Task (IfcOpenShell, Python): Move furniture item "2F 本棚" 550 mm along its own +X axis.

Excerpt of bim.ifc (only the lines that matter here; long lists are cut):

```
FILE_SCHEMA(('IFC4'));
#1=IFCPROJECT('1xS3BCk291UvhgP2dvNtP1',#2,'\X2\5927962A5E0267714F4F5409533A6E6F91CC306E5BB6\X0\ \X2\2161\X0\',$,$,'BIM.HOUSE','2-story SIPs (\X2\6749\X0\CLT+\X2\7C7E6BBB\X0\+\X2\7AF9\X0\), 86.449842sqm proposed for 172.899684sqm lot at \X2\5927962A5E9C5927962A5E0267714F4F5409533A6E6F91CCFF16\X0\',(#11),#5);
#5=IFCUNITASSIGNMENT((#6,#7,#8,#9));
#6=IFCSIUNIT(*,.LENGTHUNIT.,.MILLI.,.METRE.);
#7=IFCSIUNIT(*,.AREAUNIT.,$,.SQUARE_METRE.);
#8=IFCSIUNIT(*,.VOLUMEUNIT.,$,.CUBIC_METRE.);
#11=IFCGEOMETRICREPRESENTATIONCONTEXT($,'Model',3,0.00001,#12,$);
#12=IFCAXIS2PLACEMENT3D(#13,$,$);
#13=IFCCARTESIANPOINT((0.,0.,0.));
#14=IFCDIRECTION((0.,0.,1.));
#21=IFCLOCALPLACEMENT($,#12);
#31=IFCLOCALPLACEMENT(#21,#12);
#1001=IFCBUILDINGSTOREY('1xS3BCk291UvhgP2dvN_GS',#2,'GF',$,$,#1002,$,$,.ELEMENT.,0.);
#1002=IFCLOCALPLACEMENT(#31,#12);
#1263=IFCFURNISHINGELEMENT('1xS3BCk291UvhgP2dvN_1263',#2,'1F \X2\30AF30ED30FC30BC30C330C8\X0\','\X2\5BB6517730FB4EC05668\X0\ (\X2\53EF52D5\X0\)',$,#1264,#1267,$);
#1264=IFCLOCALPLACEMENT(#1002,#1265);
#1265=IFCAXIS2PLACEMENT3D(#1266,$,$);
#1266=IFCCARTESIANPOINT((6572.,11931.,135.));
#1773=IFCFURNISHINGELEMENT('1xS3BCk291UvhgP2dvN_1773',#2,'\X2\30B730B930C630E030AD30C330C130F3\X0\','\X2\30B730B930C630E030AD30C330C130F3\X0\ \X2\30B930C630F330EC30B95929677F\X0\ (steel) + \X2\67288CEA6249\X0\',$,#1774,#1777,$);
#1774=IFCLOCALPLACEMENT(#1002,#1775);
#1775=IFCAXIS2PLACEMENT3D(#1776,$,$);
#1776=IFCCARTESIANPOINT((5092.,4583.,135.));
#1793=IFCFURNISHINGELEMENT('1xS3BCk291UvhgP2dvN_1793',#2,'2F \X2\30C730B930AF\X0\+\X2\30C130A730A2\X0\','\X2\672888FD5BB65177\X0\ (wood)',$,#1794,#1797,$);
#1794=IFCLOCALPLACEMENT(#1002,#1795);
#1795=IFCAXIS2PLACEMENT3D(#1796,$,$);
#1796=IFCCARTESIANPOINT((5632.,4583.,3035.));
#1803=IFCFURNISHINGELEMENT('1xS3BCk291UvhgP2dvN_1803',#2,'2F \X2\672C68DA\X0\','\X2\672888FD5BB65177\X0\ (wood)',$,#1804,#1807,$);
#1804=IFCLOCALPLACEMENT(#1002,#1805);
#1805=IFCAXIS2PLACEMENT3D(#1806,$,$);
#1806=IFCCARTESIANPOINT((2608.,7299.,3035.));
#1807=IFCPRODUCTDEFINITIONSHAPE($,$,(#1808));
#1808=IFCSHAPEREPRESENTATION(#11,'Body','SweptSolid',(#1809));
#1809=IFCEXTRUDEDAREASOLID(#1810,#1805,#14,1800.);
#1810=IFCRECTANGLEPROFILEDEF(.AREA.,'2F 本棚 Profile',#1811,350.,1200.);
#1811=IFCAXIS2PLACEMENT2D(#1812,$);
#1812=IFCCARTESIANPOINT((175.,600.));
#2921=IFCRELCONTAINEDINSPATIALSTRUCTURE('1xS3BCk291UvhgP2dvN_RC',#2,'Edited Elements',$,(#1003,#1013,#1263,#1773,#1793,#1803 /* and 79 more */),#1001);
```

```python
import ifcopenshell
import ifcopenshell.api.geometry
import ifcopenshell.util.placement
import ifcopenshell.util.unit

model = ifcopenshell.open("bim.ifc")
unit_scale = ifcopenshell.util.unit.calculate_unit_scale(model)

item = model.by_guid("1xS3BCk291UvhgP2dvN_1803")
matrix = ifcopenshell.util.placement.get_local_placement(item.ObjectPlacement)
matrix[:3, 3] += matrix[:3, 0] * 0.55 / unit_scale
ifcopenshell.api.geometry.edit_object_placement(model, product=item, matrix=matrix, is_si=False)

print(ifcopenshell.util.placement.get_local_placement(item.ObjectPlacement).round(3) + 0.0)

model.write("bim_rev.ifc")
```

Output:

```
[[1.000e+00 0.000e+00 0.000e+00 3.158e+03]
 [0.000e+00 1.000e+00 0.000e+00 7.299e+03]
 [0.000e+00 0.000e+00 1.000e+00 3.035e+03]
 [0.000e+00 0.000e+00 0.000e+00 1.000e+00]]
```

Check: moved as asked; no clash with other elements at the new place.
